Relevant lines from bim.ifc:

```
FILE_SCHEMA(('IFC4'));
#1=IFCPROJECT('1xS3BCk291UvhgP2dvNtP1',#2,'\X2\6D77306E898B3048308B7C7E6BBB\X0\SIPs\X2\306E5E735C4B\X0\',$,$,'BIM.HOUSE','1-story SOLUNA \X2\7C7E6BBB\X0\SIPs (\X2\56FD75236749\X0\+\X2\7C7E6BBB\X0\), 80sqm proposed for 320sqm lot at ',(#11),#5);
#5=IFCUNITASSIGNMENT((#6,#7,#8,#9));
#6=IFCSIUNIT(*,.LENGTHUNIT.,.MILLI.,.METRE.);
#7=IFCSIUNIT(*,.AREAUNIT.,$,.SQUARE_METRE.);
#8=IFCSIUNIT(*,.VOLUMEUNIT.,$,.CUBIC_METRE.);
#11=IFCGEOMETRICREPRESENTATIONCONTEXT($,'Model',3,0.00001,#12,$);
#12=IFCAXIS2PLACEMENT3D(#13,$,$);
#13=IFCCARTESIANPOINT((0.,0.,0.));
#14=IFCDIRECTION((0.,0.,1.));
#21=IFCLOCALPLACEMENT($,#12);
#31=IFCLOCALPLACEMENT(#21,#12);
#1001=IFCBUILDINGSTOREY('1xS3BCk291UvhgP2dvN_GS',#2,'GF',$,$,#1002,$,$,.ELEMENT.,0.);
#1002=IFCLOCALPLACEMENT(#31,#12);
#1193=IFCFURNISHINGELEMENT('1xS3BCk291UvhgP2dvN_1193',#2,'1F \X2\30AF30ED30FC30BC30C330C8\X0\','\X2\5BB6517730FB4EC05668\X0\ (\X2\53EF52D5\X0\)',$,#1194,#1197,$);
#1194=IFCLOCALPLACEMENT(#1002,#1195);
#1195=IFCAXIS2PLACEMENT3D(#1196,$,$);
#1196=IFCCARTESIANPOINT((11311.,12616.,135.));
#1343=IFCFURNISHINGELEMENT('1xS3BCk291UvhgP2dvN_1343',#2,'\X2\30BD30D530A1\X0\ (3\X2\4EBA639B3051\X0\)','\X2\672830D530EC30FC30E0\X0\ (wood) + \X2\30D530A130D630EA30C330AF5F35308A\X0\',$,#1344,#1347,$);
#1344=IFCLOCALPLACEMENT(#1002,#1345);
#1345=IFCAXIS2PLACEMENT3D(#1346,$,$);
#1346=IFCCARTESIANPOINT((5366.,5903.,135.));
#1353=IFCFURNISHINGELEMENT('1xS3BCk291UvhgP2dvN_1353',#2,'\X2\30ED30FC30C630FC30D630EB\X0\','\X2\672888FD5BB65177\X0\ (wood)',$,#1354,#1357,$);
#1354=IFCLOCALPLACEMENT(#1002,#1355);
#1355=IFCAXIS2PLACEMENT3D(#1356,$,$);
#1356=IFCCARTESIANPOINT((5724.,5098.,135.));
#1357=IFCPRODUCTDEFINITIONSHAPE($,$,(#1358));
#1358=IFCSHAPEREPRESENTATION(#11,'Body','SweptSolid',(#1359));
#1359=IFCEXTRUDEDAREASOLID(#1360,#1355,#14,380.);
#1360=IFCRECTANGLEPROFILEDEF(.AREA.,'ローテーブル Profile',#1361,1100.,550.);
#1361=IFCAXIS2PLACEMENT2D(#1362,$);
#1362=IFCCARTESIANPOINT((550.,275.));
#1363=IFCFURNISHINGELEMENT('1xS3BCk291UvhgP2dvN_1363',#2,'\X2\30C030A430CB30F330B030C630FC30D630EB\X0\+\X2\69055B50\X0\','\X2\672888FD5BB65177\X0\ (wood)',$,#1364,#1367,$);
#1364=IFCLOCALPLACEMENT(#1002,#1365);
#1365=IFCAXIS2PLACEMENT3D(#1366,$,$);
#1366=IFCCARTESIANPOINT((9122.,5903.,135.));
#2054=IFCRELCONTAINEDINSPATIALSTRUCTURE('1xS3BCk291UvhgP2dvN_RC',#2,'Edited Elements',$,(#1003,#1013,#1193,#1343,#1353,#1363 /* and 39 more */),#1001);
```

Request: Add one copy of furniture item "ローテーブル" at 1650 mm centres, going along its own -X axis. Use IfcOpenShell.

```python
import ifcopenshell
import ifcopenshell.api.geometry
import ifcopenshell.api.root
import ifcopenshell.util.element
import ifcopenshell.util.placement

model = ifcopenshell.open("bim.ifc")


def reuse_history(source, copy):
    """copy_class also copies each property set's owner history, people and application; keep the originals."""
    for rel in copy.IsDefinedBy:
        if rel.is_a("IfcRelDefinesByProperties") and (history := rel.RelatingPropertyDefinition.OwnerHistory):
            rel.RelatingPropertyDefinition.OwnerHistory = source.OwnerHistory
            ifcopenshell.util.element.remove_deep2(model, history)


source = model.by_guid("1xS3BCk291UvhgP2dvN_1353")
base = ifcopenshell.util.placement.get_local_placement(source.ObjectPlacement)
step = -base[:3, 0] * 1650.0

for i in range(1, 2):
    copy = ifcopenshell.api.root.copy_class(model, product=source)
    copy.Representation = ifcopenshell.util.element.copy_deep(
        model, source.Representation, exclude=["IfcGeometricRepresentationContext", "IfcRepresentationMap"]
    )
    reuse_history(source, copy)
    matrix = base.copy()
    matrix[:3, 3] += i * step
    print("added at", matrix[:3, 3].round(3) + 0.0)
    ifcopenshell.api.geometry.edit_object_placement(model, product=copy, matrix=matrix, is_si=False)

model.write("bim_v2.ifc")
```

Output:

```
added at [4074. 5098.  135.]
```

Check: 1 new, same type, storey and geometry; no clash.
